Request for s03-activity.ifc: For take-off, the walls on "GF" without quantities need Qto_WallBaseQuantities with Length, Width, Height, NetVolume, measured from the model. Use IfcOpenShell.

First a look at what the model holds.

```python
import ifcopenshell
import ifcopenshell.util.element
import ifcopenshell.util.unit

model = ifcopenshell.open("s03-activity.ifc")
print(model.schema)
for unit_type in ("LENGTHUNIT", "AREAUNIT", "VOLUMEUNIT"):
    print(unit_type, ifcopenshell.util.unit.calculate_unit_scale(model, unit_type))
storey = next(s for s in model.by_type("IfcBuildingStorey") if s.Name == "GF")
walls = [e for e in ifcopenshell.util.element.get_decomposition(storey) if e.is_a("IfcWall")]
for e in sorted(walls, key=lambda e: e.id()):
    print(e.id(), e.is_a(), e.Name, list(ifcopenshell.util.element.get_psets(e, qtos_only=True)), sep=" | ")
```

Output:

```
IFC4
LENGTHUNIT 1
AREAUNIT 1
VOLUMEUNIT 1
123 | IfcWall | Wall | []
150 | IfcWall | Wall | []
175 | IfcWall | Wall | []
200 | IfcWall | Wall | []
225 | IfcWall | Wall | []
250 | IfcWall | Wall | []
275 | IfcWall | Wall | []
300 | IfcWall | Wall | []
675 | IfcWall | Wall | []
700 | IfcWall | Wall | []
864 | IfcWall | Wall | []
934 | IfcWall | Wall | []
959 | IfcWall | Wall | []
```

```python
import ifcopenshell
import ifcopenshell.api.pset
import ifcopenshell.geom
import ifcopenshell.util.element
import ifcopenshell.util.shape
import ifcopenshell.util.unit

model = ifcopenshell.open("s03-activity.ifc")
unit_scale = ifcopenshell.util.unit.calculate_unit_scale(model)
volume_scale = ifcopenshell.util.unit.calculate_unit_scale(model, "VOLUMEUNIT")
settings = ifcopenshell.geom.settings()

storey = next(s for s in model.by_type("IfcBuildingStorey") if s.Name == "GF")
walls = [e for e in ifcopenshell.util.element.get_decomposition(storey) if e.is_a("IfcWall")]

for e in sorted(walls, key=lambda e: e.id()):
    if ifcopenshell.util.element.get_psets(e, qtos_only=True, should_inherit=False):
        continue
    # Geometry comes back in metres, in the element's own axes.
    shape = ifcopenshell.geom.create_shape(settings, e)
    values = {
        "Length": ifcopenshell.util.shape.get_x(shape.geometry) / unit_scale,
        "Width": ifcopenshell.util.shape.get_y(shape.geometry) / unit_scale,
        "Height": ifcopenshell.util.shape.get_z(shape.geometry) / unit_scale,
        "NetVolume": ifcopenshell.util.shape.get_volume(shape.geometry) / volume_scale,
    }
    qto = ifcopenshell.api.pset.add_qto(model, product=e, name="Qto_WallBaseQuantities")
    ifcopenshell.api.pset.edit_qto(model, qto=qto, properties=values)
    print(e.id(), {k: round(v, 3) for k, v in values.items()})

model.write("s03-activity_updated.ifc")
```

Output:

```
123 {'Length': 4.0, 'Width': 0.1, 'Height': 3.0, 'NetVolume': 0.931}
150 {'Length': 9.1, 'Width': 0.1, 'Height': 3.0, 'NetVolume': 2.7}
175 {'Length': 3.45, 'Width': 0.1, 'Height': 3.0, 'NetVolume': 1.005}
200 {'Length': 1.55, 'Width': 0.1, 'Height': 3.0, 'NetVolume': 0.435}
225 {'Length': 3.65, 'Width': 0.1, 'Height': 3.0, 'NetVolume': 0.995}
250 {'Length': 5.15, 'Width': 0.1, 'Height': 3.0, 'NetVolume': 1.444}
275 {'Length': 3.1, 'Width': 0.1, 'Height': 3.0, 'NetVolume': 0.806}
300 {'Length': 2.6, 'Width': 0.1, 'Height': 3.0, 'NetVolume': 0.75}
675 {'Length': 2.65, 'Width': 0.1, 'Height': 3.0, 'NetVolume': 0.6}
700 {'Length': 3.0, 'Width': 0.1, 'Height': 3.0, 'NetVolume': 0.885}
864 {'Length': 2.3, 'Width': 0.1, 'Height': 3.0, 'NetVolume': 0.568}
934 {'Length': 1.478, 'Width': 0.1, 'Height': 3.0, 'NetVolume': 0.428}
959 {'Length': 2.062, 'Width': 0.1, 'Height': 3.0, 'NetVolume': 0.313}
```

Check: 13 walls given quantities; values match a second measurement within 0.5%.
